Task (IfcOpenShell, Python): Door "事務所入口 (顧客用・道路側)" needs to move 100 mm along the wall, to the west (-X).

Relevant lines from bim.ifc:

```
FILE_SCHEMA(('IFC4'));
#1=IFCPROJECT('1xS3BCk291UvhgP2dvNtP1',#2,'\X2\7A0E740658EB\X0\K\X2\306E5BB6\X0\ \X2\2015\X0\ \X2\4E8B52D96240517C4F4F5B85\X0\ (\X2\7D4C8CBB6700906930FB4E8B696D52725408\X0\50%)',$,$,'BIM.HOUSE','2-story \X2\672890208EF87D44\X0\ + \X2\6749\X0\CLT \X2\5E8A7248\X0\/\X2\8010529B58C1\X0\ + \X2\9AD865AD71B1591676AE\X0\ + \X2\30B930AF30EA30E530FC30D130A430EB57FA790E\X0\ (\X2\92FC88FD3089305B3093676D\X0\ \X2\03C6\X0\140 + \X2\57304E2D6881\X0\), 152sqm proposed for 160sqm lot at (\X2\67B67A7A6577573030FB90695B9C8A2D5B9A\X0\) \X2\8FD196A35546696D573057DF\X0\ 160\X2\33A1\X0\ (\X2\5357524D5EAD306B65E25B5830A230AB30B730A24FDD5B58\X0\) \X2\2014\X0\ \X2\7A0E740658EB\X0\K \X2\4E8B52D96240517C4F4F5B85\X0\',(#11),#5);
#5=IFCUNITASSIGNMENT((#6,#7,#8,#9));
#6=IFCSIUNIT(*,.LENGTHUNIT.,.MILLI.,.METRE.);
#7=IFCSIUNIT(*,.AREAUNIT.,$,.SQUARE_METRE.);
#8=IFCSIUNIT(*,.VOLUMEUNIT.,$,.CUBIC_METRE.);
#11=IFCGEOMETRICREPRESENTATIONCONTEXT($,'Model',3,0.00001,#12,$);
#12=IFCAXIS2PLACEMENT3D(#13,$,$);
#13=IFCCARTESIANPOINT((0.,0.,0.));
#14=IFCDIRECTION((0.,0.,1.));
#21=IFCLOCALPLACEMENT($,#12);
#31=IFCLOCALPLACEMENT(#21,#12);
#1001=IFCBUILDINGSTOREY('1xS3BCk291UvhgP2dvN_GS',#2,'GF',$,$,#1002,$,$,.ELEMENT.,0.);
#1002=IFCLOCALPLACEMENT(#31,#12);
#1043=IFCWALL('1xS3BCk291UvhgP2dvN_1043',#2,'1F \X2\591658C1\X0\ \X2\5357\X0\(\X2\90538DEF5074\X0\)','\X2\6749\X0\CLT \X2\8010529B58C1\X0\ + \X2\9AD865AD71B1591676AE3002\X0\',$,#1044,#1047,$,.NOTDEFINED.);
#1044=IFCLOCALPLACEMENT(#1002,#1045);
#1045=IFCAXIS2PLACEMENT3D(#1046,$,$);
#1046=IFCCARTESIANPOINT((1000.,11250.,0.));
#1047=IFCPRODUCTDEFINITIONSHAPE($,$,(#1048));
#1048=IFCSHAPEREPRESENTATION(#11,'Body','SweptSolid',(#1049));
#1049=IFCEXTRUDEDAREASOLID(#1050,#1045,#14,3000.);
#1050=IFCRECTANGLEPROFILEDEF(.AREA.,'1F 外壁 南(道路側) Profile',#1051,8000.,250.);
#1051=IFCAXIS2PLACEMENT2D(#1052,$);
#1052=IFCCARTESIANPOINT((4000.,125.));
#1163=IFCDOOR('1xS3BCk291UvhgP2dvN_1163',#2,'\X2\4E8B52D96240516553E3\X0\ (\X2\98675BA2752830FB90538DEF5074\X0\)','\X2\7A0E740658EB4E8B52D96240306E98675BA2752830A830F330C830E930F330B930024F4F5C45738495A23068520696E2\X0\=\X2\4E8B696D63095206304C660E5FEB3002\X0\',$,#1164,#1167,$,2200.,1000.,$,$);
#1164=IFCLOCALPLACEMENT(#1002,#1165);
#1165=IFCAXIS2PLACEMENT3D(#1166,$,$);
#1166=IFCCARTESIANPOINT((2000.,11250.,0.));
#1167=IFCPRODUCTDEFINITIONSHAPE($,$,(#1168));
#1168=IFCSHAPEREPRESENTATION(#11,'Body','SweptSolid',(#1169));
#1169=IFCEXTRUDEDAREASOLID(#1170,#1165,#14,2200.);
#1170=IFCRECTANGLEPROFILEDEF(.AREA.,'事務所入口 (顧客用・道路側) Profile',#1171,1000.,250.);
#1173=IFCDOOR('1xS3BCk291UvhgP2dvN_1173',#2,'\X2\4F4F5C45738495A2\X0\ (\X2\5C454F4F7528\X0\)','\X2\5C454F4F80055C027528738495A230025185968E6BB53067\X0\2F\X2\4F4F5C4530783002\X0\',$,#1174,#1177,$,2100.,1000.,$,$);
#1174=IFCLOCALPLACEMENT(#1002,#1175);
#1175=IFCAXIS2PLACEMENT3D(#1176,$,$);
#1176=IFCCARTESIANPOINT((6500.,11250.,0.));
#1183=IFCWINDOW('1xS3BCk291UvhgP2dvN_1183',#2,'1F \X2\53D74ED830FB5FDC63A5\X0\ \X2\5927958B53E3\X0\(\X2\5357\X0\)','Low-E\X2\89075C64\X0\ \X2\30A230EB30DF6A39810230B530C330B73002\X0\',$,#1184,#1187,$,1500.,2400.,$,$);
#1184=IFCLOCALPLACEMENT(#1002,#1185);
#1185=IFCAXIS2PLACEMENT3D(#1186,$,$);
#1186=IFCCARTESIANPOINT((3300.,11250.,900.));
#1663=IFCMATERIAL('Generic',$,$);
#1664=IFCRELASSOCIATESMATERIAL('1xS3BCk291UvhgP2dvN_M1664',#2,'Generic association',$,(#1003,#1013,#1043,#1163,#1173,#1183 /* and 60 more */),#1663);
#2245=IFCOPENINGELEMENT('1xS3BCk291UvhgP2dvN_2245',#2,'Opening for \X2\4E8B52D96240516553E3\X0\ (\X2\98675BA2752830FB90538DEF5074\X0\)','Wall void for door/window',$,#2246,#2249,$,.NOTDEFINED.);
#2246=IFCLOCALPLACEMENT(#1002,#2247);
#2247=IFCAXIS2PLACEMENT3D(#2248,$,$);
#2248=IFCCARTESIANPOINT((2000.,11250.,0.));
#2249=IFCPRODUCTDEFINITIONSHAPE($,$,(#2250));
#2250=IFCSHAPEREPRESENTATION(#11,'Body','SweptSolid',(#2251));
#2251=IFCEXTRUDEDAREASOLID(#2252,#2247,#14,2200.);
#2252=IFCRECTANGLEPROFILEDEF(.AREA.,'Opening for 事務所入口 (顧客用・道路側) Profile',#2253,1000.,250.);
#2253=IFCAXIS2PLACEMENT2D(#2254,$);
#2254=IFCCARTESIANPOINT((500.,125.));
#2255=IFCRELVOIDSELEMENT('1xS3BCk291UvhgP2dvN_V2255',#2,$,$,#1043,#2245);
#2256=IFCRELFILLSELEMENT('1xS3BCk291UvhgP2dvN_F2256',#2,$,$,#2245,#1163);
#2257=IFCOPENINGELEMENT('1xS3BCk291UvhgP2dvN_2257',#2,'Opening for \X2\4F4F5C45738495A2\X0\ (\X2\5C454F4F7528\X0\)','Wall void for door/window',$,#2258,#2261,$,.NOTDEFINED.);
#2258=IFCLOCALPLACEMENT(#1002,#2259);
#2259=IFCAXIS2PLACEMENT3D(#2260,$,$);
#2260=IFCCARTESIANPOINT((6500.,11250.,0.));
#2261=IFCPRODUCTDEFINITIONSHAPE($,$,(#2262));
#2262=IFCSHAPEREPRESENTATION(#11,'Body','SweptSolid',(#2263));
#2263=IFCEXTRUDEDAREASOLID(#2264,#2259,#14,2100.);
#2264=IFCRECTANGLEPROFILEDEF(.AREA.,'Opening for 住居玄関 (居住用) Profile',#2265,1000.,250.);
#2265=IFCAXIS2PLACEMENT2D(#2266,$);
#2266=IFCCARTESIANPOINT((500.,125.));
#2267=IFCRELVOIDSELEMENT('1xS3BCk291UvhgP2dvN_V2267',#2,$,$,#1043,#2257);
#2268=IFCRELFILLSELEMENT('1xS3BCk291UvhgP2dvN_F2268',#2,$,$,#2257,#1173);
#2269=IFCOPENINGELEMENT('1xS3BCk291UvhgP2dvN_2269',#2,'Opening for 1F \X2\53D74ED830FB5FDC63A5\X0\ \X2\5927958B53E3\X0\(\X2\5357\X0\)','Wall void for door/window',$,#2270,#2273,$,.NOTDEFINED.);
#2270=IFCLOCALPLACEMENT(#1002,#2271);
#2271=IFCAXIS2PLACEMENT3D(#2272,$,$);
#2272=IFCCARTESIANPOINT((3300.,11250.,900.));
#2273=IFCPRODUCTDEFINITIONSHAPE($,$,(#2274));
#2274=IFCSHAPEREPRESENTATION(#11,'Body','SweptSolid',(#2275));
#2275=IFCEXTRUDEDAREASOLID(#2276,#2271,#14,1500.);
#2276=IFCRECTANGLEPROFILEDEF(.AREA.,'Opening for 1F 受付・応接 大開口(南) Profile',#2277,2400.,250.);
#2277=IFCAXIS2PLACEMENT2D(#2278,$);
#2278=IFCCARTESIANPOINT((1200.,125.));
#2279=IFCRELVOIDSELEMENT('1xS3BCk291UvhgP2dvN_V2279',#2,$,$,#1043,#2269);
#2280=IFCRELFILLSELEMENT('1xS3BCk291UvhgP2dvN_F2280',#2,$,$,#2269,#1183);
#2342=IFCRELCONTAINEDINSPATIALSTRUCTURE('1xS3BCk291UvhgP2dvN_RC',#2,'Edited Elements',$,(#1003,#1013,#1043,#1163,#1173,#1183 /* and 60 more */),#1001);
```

```python
import ifcopenshell
import ifcopenshell.api.geometry
import ifcopenshell.util.placement
import ifcopenshell.util.unit

model = ifcopenshell.open("bim.ifc")
unit_scale = ifcopenshell.util.unit.calculate_unit_scale(model)

door = model.by_guid("1xS3BCk291UvhgP2dvN_1163")
opening = door.FillsVoids[0].RelatingOpeningElement
wall = opening.VoidsElements[0].RelatingBuildingElement

wall_matrix = ifcopenshell.util.placement.get_local_placement(wall.ObjectPlacement)
shift = wall_matrix[:3, 0] * -0.1 / unit_scale
before = ifcopenshell.util.placement.get_local_placement(door.ObjectPlacement)[:3, 3].copy()

# The door is not placed relative to its opening, so move both.
for product in (opening, door):
    matrix = ifcopenshell.util.placement.get_local_placement(product.ObjectPlacement)
    matrix[:3, 3] += shift
    ifcopenshell.api.geometry.edit_object_placement(model, product=product, matrix=matrix, is_si=False)

after = ifcopenshell.util.placement.get_local_placement(door.ObjectPlacement)[:3, 3]
print("door moved by", (after - before).round(3) + 0.0)

model.write("bim_edited.ifc")
```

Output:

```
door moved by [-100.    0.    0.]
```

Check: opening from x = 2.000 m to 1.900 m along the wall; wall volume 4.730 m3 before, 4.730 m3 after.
